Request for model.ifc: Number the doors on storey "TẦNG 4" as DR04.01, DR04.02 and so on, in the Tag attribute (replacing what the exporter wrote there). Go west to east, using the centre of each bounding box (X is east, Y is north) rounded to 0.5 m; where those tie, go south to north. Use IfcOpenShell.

First a look at what the model holds.

```python
import ifcopenshell
import ifcopenshell.util.element
import ifcopenshell.util.placement

model = ifcopenshell.open("model.ifc")
print(model.schema)
storey = next(s for s in model.by_type("IfcBuildingStorey") if s.Name == "TẦNG 4")
doors = [e for e in ifcopenshell.util.element.get_decomposition(storey) if e.is_a("IfcDoor")]
for e in sorted(doors, key=lambda e: e.id()):
    origin = ifcopenshell.util.placement.get_local_placement(e.ObjectPlacement)[:3, 3]
    print(e.id(), e.Tag, e.Name, origin.round(2) + 0.0, sep=" | ")
```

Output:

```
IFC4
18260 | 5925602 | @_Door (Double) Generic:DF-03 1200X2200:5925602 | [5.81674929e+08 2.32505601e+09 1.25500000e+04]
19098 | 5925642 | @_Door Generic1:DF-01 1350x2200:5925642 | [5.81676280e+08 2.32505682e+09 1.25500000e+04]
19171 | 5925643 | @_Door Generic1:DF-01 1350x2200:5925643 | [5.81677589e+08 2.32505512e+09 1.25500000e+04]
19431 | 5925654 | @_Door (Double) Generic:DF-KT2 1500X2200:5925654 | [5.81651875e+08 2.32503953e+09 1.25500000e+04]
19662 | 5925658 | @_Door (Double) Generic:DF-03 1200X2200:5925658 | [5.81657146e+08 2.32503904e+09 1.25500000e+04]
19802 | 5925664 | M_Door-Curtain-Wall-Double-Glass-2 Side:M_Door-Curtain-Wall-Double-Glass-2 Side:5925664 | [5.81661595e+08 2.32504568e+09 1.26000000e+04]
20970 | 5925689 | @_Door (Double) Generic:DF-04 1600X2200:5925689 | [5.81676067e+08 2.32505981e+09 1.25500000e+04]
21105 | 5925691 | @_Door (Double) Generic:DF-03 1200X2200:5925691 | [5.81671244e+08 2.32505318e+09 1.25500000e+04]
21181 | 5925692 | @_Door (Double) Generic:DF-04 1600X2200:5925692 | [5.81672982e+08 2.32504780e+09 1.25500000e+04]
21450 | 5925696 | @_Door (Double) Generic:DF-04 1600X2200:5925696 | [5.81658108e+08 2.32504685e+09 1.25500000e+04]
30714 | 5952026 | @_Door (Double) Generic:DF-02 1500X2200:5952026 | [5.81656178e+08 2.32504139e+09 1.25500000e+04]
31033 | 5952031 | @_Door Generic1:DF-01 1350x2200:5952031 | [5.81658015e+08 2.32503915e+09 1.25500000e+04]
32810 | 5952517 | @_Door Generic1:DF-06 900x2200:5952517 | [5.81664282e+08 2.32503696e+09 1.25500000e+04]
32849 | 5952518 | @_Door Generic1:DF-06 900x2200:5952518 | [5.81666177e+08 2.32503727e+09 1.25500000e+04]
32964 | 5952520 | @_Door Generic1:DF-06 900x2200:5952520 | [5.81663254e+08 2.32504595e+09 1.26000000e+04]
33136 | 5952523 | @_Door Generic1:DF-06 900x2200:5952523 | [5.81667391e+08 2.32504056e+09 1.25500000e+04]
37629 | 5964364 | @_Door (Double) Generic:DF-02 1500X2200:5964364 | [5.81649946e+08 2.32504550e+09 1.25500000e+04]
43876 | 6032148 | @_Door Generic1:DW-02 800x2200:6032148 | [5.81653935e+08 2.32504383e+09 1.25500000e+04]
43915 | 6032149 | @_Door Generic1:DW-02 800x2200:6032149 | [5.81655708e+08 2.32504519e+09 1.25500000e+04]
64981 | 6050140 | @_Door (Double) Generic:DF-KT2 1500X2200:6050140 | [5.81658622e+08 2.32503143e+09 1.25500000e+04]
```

```python
import ifcopenshell
import ifcopenshell.geom
import ifcopenshell.util.element
import ifcopenshell.util.shape

model = ifcopenshell.open("model.ifc")
settings = ifcopenshell.geom.settings()
settings.set("use-world-coords", True)


def centre(element):
    shape = ifcopenshell.geom.create_shape(settings, element)
    return ifcopenshell.util.shape.get_bbox_centroid(shape.geometry)


storey = next(s for s in model.by_type("IfcBuildingStorey") if s.Name == "TẦNG 4")
doors = [e for e in ifcopenshell.util.element.get_decomposition(storey) if e.is_a("IfcDoor")]

# Insertion points can sit at a corner or the storey origin, so sort by the geometry (in metres).
centres = {e: centre(e) for e in doors}
doors.sort(key=lambda e: (round(centres[e][0] / 0.5), centres[e][1]))

for i, e in enumerate(doors, start=1):
    number = f"DR04.{i:02d}"
    e.Tag = number
    print(e.id(), number)

model.write("model_edited.ifc")
```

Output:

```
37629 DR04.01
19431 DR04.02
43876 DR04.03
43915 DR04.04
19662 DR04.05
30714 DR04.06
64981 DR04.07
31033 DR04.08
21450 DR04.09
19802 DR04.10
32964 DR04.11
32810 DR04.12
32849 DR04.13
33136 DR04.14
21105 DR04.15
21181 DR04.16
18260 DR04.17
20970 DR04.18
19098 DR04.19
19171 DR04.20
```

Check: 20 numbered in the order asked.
